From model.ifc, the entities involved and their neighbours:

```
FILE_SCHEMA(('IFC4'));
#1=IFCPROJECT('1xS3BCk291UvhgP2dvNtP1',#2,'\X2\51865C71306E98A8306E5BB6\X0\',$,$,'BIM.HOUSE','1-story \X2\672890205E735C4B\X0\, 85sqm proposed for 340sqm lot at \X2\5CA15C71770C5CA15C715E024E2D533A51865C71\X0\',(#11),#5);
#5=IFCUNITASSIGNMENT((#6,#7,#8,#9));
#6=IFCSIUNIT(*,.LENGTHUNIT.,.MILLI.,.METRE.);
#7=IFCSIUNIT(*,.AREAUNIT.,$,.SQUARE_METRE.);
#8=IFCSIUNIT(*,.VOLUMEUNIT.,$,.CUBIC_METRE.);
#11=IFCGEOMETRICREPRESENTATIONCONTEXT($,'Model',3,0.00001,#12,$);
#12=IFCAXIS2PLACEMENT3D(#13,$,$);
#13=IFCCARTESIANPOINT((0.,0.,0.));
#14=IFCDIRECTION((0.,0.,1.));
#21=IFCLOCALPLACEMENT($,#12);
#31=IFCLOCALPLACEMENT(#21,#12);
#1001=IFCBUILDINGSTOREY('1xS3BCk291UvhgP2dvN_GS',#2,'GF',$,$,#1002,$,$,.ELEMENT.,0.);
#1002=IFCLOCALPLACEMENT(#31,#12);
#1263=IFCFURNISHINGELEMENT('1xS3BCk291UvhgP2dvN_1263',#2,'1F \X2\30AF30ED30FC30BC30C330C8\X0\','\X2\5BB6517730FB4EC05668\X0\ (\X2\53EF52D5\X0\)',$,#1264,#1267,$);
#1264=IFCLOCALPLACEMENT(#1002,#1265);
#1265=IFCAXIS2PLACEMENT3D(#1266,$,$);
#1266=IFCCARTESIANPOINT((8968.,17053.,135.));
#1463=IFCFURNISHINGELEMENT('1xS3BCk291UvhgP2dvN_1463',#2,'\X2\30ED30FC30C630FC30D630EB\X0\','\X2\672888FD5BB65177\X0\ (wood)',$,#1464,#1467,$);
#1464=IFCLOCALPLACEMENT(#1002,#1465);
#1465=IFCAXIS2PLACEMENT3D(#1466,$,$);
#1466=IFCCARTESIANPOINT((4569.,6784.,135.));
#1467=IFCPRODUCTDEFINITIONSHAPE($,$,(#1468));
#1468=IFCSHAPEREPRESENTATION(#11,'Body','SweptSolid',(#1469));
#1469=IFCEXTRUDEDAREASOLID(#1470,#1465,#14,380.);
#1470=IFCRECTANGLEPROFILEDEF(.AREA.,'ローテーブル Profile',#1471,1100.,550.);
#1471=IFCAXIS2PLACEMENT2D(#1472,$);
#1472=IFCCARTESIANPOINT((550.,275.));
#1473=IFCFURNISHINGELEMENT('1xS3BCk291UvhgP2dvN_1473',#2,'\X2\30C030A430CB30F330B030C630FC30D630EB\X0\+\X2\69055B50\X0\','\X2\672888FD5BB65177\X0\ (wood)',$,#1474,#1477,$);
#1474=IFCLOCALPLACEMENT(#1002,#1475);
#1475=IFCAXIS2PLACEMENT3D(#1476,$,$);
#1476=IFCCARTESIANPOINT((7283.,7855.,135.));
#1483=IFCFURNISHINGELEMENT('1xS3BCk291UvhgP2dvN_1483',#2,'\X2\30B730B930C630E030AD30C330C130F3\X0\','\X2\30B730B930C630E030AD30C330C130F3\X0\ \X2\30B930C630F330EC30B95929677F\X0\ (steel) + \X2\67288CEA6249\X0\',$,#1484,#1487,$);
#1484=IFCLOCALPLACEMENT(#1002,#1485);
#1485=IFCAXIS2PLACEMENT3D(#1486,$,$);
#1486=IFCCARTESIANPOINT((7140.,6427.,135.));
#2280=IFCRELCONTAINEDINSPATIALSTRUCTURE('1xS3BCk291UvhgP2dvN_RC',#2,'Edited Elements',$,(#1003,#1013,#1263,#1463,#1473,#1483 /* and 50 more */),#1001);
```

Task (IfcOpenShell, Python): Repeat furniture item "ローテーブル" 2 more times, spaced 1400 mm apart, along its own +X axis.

```python
import ifcopenshell
import ifcopenshell.api.geometry
import ifcopenshell.api.root
import ifcopenshell.util.element
import ifcopenshell.util.placement
import ifcopenshell.util.unit

model = ifcopenshell.open("model.ifc")
unit_scale = ifcopenshell.util.unit.calculate_unit_scale(model)


def reuse_history(source, copy):
    """copy_class also copies each property set's owner history, people and application; keep the originals."""
    for rel in copy.IsDefinedBy:
        if rel.is_a("IfcRelDefinesByProperties") and (history := rel.RelatingPropertyDefinition.OwnerHistory):
            rel.RelatingPropertyDefinition.OwnerHistory = source.OwnerHistory
            ifcopenshell.util.element.remove_deep2(model, history)


source = model.by_id(1463)
base = ifcopenshell.util.placement.get_local_placement(source.ObjectPlacement)
step = base[:3, 0] * 1.4 / unit_scale

for i in range(1, 3):
    copy = ifcopenshell.api.root.copy_class(model, product=source)
    copy.Representation = ifcopenshell.util.element.copy_deep(
        model, source.Representation, exclude=["IfcGeometricRepresentationContext", "IfcRepresentationMap"]
    )
    reuse_history(source, copy)
    matrix = base.copy()
    matrix[:3, 3] += i * step
    print("added at", matrix[:3, 3].round(3) + 0.0)
    ifcopenshell.api.geometry.edit_object_placement(model, product=copy, matrix=matrix, is_si=False)

model.write("model_v2.ifc")
```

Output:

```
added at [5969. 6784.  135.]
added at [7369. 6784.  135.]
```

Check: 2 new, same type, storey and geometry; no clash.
